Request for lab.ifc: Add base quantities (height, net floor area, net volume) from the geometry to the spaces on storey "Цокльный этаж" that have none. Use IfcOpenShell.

First a look at what the model holds.

```python
import ifcopenshell
import ifcopenshell.util.element
import ifcopenshell.util.unit

model = ifcopenshell.open("lab.ifc")
print(model.schema)
for unit_type in ("LENGTHUNIT", "AREAUNIT", "VOLUMEUNIT"):
    print(unit_type, ifcopenshell.util.unit.calculate_unit_scale(model, unit_type))
storey = next(s for s in model.by_type("IfcBuildingStorey") if s.Name == "Цокльный этаж")
spaces = [e for e in ifcopenshell.util.element.get_decomposition(storey) if e.is_a("IfcSpace")]
for e in sorted(spaces, key=lambda e: e.id()):
    print(e.id(), e.is_a(), e.Name, list(ifcopenshell.util.element.get_psets(e, qtos_only=True)), sep=" | ")
```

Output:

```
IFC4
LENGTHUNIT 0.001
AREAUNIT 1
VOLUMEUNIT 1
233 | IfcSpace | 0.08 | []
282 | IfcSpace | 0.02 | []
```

```python
import ifcopenshell
import ifcopenshell.api.pset
import ifcopenshell.geom
import ifcopenshell.util.element
import ifcopenshell.util.shape
import ifcopenshell.util.unit

model = ifcopenshell.open("lab.ifc")
unit_scale = ifcopenshell.util.unit.calculate_unit_scale(model)
area_scale = ifcopenshell.util.unit.calculate_unit_scale(model, "AREAUNIT")
volume_scale = ifcopenshell.util.unit.calculate_unit_scale(model, "VOLUMEUNIT")
settings = ifcopenshell.geom.settings()

storey = next(s for s in model.by_type("IfcBuildingStorey") if s.Name == "Цокльный этаж")
spaces = [e for e in ifcopenshell.util.element.get_decomposition(storey) if e.is_a("IfcSpace")]

for e in sorted(spaces, key=lambda e: e.id()):
    if ifcopenshell.util.element.get_psets(e, qtos_only=True, should_inherit=False):
        continue
    # Geometry comes back in metres, in the element's own axes.
    shape = ifcopenshell.geom.create_shape(settings, e)
    values = {
        "Height": ifcopenshell.util.shape.get_z(shape.geometry) / unit_scale,
        "NetFloorArea": ifcopenshell.util.shape.get_footprint_area(shape.geometry) / area_scale,
        "NetVolume": ifcopenshell.util.shape.get_volume(shape.geometry) / volume_scale,
    }
    qto = ifcopenshell.api.pset.add_qto(model, product=e, name="Qto_SpaceBaseQuantities")
    ifcopenshell.api.pset.edit_qto(model, qto=qto, properties=values)
    print(e.id(), {k: round(v, 3) for k, v in values.items()})

model.write("lab_updated.ifc")
```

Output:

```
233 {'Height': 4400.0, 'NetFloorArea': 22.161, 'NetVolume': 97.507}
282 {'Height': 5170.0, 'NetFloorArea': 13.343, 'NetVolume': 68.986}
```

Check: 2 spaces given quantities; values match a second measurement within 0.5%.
